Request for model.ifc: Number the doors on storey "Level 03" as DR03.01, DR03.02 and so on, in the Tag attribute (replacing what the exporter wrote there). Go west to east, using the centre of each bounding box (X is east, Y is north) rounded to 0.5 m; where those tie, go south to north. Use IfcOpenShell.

First a look at what the model holds.

```python
import ifcopenshell
import ifcopenshell.util.element
import ifcopenshell.util.placement

model = ifcopenshell.open("model.ifc")
print(model.schema)
storey = next(s for s in model.by_type("IfcBuildingStorey") if s.Name == "Level 03")
doors = [e for e in ifcopenshell.util.element.get_decomposition(storey) if e.is_a("IfcDoor")]
for e in sorted(doors, key=lambda e: e.id()):
    origin = ifcopenshell.util.placement.get_local_placement(e.ObjectPlacement)[:3, 3]
    print(e.id(), e.Tag, e.Name, origin.round(2) + 0.0, sep=" | ")
```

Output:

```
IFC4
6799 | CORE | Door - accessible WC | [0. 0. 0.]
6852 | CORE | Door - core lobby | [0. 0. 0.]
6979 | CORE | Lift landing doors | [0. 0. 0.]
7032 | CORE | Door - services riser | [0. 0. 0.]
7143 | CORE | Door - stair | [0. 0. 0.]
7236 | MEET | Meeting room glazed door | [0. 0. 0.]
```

```python
import ifcopenshell
import ifcopenshell.geom
import ifcopenshell.util.element
import ifcopenshell.util.shape

model = ifcopenshell.open("model.ifc")
settings = ifcopenshell.geom.settings()
settings.set("use-world-coords", True)


def centre(element):
    shape = ifcopenshell.geom.create_shape(settings, element)
    return ifcopenshell.util.shape.get_bbox_centroid(shape.geometry)


storey = next(s for s in model.by_type("IfcBuildingStorey") if s.Name == "Level 03")
doors = [e for e in ifcopenshell.util.element.get_decomposition(storey) if e.is_a("IfcDoor")]

# Insertion points can sit at a corner or the storey origin, so sort by the geometry (in metres).
centres = {e: centre(e) for e in doors}
doors.sort(key=lambda e: (round(centres[e][0] / 0.5), centres[e][1]))

for i, e in enumerate(doors, start=1):
    number = f"DR03.{i:02d}"
    e.Tag = number
    print(e.id(), number)

model.write("model-out.ifc")
```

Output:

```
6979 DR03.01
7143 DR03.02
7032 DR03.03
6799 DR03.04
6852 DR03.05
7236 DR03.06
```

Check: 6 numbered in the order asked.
